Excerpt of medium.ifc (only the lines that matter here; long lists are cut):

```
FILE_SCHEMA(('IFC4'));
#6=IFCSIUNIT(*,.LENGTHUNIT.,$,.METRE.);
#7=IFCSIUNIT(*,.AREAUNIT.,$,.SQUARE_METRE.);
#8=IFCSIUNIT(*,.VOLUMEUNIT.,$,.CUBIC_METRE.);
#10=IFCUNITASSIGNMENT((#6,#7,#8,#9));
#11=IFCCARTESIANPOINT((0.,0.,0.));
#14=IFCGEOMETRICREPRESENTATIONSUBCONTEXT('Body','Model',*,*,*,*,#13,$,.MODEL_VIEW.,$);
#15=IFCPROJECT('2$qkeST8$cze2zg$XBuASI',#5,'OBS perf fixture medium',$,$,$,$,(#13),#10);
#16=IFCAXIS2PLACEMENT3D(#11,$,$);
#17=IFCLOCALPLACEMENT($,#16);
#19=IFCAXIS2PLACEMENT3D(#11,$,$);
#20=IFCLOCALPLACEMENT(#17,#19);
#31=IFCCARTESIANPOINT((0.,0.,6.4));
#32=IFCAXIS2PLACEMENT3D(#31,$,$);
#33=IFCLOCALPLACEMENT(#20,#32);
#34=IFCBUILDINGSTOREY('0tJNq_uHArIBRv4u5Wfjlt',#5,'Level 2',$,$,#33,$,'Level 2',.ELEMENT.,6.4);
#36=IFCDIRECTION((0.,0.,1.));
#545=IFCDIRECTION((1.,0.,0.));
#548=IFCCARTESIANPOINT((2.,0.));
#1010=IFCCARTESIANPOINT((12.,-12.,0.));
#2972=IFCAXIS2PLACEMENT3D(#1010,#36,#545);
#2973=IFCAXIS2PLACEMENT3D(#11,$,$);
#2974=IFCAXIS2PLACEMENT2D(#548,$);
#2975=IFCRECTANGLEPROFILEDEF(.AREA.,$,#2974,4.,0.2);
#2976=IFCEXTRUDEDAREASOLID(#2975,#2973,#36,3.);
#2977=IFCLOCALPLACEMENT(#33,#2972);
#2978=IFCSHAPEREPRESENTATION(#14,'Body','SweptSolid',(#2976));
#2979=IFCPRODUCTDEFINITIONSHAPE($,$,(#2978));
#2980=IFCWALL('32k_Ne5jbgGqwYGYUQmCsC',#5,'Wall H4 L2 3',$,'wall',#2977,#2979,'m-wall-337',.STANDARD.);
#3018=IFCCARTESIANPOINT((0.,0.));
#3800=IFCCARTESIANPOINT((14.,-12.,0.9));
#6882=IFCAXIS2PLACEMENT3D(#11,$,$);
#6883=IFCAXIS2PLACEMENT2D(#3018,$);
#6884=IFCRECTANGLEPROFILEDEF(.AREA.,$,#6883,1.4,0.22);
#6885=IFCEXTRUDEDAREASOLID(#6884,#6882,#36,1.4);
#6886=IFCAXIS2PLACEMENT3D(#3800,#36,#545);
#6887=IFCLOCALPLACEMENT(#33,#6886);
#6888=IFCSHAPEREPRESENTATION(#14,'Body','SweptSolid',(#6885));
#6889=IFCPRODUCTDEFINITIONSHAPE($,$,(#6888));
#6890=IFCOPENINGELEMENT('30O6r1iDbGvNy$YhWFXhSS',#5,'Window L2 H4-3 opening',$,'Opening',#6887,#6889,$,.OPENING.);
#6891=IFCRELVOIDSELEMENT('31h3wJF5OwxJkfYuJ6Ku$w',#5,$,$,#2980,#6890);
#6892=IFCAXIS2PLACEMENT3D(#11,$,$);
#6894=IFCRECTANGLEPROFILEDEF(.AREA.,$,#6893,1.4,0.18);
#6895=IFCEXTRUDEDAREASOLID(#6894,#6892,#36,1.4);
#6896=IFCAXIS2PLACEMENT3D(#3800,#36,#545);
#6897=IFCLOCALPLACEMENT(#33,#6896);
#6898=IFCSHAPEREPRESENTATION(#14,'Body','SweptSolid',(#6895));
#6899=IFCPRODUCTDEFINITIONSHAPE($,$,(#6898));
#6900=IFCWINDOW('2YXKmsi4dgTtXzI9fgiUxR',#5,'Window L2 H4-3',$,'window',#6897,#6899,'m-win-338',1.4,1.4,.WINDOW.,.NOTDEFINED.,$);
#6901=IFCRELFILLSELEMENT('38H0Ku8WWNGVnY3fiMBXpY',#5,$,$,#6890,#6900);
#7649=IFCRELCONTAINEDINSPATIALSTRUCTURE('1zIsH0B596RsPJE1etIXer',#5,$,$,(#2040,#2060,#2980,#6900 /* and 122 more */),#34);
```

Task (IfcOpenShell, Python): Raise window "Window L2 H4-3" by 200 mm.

```python
import numpy as np
import ifcopenshell
import ifcopenshell.api.geometry
import ifcopenshell.util.placement
import ifcopenshell.util.unit

model = ifcopenshell.open("medium.ifc")
unit_scale = ifcopenshell.util.unit.calculate_unit_scale(model)

window = model.by_guid("2YXKmsi4dgTtXzI9fgiUxR")
opening = window.FillsVoids[0].RelatingOpeningElement
dz = 0.2 / unit_scale

shift = np.array([0.0, 0.0, dz])
# The window is not placed relative to its opening, so move both.
for product in (opening, window):
    matrix = ifcopenshell.util.placement.get_local_placement(product.ObjectPlacement)
    matrix[:3, 3] += shift
    ifcopenshell.api.geometry.edit_object_placement(model, product=product, matrix=matrix, is_si=False)

print(f"moved by {dz * unit_scale:+.3f} m")

model.write("medium_v2.ifc")
```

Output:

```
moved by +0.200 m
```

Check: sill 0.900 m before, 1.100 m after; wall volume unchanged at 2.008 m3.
